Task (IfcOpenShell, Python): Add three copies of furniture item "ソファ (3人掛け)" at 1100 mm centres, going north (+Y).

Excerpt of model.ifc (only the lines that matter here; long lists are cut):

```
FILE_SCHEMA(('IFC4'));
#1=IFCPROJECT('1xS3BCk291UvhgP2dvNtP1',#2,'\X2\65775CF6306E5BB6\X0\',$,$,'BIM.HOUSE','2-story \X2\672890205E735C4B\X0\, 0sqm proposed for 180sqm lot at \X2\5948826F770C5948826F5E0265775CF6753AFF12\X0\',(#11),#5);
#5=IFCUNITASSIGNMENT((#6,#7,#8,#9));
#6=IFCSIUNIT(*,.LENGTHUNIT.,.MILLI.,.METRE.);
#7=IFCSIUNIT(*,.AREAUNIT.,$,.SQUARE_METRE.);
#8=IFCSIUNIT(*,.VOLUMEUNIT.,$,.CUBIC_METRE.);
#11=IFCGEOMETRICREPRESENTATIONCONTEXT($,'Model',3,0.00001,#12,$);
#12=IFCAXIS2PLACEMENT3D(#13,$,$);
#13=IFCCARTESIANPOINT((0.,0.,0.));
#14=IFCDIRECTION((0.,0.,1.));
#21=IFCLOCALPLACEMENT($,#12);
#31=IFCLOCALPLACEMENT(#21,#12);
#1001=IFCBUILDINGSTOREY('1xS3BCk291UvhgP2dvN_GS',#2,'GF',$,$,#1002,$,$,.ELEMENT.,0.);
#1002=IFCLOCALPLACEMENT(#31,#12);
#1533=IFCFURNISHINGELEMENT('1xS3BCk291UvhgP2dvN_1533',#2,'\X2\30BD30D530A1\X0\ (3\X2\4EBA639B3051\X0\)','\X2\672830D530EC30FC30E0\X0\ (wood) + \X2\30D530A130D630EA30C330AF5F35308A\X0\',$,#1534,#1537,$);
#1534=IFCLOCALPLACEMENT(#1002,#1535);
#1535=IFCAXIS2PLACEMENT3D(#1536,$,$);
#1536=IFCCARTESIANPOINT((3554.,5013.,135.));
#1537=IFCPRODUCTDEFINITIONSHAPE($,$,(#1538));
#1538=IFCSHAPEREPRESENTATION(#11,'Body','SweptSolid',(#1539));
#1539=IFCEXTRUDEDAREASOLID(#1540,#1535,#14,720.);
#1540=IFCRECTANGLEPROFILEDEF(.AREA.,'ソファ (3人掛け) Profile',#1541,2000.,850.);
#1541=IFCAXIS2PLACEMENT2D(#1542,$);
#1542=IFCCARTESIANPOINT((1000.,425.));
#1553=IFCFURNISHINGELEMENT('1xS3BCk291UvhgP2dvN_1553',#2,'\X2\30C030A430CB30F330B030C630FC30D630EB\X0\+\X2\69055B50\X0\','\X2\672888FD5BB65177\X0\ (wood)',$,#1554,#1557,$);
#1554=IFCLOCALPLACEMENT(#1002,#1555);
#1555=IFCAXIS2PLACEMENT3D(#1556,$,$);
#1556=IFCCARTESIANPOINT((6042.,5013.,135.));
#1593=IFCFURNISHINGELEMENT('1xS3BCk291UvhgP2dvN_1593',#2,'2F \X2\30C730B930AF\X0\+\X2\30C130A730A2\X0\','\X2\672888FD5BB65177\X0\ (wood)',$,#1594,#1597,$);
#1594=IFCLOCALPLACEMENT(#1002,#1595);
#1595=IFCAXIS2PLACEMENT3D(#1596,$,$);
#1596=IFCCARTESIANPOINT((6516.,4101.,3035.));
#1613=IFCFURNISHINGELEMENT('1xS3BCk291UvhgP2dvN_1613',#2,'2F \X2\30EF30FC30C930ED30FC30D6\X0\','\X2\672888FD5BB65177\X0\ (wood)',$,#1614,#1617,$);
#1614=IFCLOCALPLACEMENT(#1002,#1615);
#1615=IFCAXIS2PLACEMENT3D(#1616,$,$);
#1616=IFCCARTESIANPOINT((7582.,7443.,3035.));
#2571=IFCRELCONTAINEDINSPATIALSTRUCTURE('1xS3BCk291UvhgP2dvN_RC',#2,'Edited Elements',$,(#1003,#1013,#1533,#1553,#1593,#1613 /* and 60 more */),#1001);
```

```python
import numpy as np
import ifcopenshell
import ifcopenshell.api.geometry
import ifcopenshell.api.root
import ifcopenshell.util.element
import ifcopenshell.util.placement

model = ifcopenshell.open("model.ifc")


def reuse_history(source, copy):
    """copy_class also copies each property set's owner history, people and application; keep the originals."""
    for rel in copy.IsDefinedBy:
        if rel.is_a("IfcRelDefinesByProperties") and (history := rel.RelatingPropertyDefinition.OwnerHistory):
            rel.RelatingPropertyDefinition.OwnerHistory = source.OwnerHistory
            ifcopenshell.util.element.remove_deep2(model, history)


source = model.by_guid("1xS3BCk291UvhgP2dvN_1533")
base = ifcopenshell.util.placement.get_local_placement(source.ObjectPlacement)
step = np.array([0.0, 1.0, 0.0]) * 1100.0

for i in range(1, 4):
    copy = ifcopenshell.api.root.copy_class(model, product=source)
    copy.Representation = ifcopenshell.util.element.copy_deep(
        model, source.Representation, exclude=["IfcGeometricRepresentationContext", "IfcRepresentationMap"]
    )
    reuse_history(source, copy)
    matrix = base.copy()
    matrix[:3, 3] += i * step
    print("added at", matrix[:3, 3].round(3) + 0.0)
    ifcopenshell.api.geometry.edit_object_placement(model, product=copy, matrix=matrix, is_si=False)

model.write("model_v2.ifc")
```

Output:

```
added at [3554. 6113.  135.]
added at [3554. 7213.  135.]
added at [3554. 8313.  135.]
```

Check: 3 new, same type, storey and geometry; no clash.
